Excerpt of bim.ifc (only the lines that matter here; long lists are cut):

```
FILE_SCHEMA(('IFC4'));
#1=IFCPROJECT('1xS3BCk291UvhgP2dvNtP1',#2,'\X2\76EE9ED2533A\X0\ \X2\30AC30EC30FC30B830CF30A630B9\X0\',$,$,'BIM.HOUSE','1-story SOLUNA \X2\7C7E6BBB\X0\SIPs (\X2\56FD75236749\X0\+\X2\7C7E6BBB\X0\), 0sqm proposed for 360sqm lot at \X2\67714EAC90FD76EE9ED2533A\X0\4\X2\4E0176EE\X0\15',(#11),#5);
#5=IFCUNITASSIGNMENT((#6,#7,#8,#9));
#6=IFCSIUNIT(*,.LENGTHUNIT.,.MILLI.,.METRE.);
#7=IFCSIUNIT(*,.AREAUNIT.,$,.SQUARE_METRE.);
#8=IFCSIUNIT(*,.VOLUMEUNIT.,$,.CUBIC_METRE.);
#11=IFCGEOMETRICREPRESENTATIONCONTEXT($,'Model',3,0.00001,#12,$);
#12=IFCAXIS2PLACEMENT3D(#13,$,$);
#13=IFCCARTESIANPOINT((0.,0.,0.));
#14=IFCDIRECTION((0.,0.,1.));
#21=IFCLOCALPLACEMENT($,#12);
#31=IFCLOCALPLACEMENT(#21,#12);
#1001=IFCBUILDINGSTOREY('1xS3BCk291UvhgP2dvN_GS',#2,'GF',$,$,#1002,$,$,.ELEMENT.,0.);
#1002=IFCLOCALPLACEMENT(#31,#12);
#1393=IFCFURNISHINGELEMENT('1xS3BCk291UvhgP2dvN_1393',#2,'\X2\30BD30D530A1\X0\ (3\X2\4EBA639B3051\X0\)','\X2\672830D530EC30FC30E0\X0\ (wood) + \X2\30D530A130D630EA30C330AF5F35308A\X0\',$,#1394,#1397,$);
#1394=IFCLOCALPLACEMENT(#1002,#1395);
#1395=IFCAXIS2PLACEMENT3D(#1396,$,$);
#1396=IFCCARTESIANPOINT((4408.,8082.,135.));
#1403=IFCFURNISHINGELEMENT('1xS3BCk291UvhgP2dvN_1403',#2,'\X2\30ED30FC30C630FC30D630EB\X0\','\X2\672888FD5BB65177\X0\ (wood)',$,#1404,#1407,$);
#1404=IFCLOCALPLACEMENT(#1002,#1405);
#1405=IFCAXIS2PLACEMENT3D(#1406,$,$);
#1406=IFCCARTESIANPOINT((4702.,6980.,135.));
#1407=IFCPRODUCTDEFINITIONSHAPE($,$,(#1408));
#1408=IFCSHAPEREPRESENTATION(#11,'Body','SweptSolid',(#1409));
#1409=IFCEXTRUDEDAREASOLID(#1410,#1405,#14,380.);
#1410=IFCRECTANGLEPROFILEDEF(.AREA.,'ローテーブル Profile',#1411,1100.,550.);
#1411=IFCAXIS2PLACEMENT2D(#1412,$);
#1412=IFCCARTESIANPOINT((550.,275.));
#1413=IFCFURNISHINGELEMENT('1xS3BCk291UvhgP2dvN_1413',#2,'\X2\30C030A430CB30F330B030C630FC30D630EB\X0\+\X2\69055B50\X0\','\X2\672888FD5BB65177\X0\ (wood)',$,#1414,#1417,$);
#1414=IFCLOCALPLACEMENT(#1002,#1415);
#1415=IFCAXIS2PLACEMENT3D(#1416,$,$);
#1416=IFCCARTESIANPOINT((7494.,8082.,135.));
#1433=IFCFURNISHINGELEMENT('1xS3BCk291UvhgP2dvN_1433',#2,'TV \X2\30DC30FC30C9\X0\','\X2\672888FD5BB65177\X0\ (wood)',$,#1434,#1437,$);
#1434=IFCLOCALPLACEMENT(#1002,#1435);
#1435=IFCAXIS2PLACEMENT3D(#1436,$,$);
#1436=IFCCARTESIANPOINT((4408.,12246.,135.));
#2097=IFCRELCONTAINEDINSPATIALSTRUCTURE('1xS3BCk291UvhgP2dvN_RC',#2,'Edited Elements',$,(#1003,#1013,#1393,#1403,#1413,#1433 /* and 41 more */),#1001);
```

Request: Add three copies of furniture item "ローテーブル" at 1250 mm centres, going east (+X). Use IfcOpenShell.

```python
import numpy as np
import ifcopenshell
import ifcopenshell.api.geometry
import ifcopenshell.api.root
import ifcopenshell.util.element
import ifcopenshell.util.placement

model = ifcopenshell.open("bim.ifc")


def reuse_history(source, copy):
    """copy_class also copies each property set's owner history, people and application; keep the originals."""
    for rel in copy.IsDefinedBy:
        if rel.is_a("IfcRelDefinesByProperties") and (history := rel.RelatingPropertyDefinition.OwnerHistory):
            rel.RelatingPropertyDefinition.OwnerHistory = source.OwnerHistory
            ifcopenshell.util.element.remove_deep2(model, history)


source = model.by_id(1403)
base = ifcopenshell.util.placement.get_local_placement(source.ObjectPlacement)
step = np.array([1.0, 0.0, 0.0]) * 1250.0

for i in range(1, 4):
    copy = ifcopenshell.api.root.copy_class(model, product=source)
    copy.Representation = ifcopenshell.util.element.copy_deep(
        model, source.Representation, exclude=["IfcGeometricRepresentationContext", "IfcRepresentationMap"]
    )
    reuse_history(source, copy)
    matrix = base.copy()
    matrix[:3, 3] += i * step
    print("added at", matrix[:3, 3].round(3) + 0.0)
    ifcopenshell.api.geometry.edit_object_placement(model, product=copy, matrix=matrix, is_si=False)

model.write("bim_v2.ifc")
```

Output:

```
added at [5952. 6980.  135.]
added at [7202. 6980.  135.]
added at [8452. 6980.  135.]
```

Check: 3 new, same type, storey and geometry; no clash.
